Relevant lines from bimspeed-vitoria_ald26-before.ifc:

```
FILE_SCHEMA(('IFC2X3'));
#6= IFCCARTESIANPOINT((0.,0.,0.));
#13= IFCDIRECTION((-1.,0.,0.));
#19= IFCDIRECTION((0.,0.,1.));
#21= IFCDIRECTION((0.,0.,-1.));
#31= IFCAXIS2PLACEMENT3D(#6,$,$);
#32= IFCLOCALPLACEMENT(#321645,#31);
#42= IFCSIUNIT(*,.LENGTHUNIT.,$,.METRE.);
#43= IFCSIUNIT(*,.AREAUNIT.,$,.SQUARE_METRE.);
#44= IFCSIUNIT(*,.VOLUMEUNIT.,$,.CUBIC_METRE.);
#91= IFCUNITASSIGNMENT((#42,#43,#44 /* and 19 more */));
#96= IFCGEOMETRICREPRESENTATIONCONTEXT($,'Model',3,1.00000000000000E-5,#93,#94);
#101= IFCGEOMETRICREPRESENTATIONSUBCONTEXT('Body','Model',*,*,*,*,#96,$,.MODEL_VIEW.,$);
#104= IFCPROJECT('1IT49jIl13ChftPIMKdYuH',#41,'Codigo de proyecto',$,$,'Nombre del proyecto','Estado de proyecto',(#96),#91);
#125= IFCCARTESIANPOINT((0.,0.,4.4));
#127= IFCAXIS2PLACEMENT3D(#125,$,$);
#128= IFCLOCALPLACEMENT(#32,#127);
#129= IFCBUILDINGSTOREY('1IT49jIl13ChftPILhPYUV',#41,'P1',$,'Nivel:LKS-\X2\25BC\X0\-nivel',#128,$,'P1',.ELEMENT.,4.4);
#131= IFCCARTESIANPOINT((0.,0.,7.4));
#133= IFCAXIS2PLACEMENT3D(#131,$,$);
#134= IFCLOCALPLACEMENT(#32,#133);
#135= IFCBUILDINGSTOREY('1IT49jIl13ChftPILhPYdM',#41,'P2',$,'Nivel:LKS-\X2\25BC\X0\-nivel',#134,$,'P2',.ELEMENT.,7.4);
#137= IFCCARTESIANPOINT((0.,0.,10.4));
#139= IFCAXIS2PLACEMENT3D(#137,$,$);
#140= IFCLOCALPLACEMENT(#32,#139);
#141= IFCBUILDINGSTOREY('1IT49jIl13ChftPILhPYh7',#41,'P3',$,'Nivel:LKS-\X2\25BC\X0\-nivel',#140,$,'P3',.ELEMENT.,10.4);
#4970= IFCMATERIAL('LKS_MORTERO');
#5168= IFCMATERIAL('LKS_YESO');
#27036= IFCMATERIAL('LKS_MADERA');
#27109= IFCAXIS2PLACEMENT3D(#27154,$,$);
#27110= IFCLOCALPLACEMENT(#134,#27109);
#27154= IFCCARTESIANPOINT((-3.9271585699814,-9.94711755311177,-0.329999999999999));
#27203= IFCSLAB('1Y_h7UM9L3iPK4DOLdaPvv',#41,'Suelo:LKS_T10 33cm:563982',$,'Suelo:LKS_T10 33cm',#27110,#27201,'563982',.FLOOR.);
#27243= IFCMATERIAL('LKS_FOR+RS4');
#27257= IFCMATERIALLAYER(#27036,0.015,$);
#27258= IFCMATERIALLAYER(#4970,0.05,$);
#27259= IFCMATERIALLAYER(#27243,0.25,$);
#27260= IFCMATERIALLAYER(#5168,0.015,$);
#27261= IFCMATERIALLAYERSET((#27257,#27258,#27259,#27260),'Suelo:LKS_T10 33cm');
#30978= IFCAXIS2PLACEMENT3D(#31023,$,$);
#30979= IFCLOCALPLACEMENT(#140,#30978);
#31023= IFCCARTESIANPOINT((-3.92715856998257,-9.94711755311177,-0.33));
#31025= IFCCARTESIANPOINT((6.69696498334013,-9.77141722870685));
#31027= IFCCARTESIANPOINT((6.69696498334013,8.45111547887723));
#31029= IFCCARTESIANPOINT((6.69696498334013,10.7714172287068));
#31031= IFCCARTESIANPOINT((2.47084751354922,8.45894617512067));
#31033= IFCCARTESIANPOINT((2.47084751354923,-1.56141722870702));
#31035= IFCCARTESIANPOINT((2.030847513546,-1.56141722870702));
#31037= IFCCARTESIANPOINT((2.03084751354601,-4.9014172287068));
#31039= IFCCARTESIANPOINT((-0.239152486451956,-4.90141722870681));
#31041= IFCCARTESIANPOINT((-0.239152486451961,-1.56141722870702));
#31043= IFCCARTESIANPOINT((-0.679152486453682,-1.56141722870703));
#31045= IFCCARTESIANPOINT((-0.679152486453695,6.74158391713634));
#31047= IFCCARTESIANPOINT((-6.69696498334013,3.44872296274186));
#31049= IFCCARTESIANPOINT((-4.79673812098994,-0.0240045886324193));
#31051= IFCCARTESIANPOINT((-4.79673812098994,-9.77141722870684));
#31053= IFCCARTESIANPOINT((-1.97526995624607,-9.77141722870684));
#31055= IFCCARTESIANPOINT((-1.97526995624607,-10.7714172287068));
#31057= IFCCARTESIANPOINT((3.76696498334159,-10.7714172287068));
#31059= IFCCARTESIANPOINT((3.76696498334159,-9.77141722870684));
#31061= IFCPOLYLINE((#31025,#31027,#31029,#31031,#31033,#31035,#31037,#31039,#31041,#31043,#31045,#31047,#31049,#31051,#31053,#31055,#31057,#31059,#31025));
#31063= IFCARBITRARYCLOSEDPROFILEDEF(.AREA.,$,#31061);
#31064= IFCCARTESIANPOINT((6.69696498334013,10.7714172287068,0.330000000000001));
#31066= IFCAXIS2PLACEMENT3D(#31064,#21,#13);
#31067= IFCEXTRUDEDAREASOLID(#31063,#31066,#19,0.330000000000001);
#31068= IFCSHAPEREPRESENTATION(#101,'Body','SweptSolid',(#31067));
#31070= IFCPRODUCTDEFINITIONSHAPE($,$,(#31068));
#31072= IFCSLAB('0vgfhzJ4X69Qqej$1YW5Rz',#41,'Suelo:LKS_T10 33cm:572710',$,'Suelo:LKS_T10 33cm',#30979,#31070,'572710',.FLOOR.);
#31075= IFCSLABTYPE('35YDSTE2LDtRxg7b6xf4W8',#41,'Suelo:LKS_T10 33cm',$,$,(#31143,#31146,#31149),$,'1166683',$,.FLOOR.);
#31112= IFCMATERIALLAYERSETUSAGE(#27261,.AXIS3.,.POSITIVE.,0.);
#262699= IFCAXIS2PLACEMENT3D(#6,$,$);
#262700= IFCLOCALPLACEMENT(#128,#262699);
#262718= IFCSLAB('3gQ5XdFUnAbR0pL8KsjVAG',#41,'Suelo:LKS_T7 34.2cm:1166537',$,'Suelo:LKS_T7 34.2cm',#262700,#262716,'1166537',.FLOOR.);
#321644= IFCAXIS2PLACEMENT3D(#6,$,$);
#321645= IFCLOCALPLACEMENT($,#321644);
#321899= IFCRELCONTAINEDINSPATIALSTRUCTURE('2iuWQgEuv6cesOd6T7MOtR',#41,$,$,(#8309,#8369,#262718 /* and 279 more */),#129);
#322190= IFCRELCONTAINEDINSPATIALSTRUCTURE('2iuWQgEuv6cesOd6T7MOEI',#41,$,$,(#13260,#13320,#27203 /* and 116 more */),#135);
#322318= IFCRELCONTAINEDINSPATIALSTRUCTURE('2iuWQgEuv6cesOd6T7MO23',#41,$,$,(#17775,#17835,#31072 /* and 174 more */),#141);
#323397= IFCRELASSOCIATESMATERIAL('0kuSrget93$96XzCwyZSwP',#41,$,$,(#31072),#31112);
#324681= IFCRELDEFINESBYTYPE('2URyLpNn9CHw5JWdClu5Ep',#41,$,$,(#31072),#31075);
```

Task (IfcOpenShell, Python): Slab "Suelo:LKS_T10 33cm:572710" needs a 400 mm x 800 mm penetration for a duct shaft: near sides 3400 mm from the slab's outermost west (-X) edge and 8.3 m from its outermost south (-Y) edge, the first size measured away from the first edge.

```python
import numpy as np
import ifcopenshell
import ifcopenshell.api.feature
import ifcopenshell.api.geometry
import ifcopenshell.api.root
import ifcopenshell.geom
import ifcopenshell.util.placement
import ifcopenshell.util.representation
import ifcopenshell.util.shape
import ifcopenshell.util.unit

model = ifcopenshell.open("bimspeed-vitoria_ald26-before.ifc")
unit_scale = ifcopenshell.util.unit.calculate_unit_scale(model)
settings = ifcopenshell.geom.settings()


def volume(element):
    """Net volume in cubic metres, openings subtracted."""
    shape = ifcopenshell.geom.create_shape(settings, element)
    return ifcopenshell.util.shape.get_volume(shape.geometry)


slab = model.by_id(31072)
before = volume(slab)

# Extent in the slab's own axes, in metres. The edges named are its -X and -Y sides.
slab_shape = ifcopenshell.geom.create_shape(settings, slab)
vertices = ifcopenshell.util.shape.get_vertices(slab_shape.geometry)
x_min, y_min, bottom = vertices.min(axis=0)
top = vertices[:, 2].max()

opening = ifcopenshell.api.root.create_entity(model, ifc_class="IfcOpeningElement", name="Duct shaft opening")
context = ifcopenshell.util.representation.get_context(model, "Model", "Body", "MODEL_VIEW")
width, depth = 0.4, 0.8
outline = [(0.0, 0.0), (width, 0.0), (width, depth), (0.0, depth), (0.0, 0.0)]
# Overshoot both faces by 50 mm so the cut is clean.
shape = ifcopenshell.api.geometry.add_slab_representation(
    model, context=context, depth=top - bottom + 0.1, polyline=outline
)
ifcopenshell.api.geometry.assign_representation(model, product=opening, representation=shape)

matrix = ifcopenshell.util.placement.get_local_placement(slab.ObjectPlacement)
matrix[:, 3] = matrix @ np.append(np.array([x_min + 3.4, y_min + 8.3, bottom - 0.05]) / unit_scale, 1.0)
ifcopenshell.api.geometry.edit_object_placement(model, product=opening, matrix=matrix, is_si=False)
ifcopenshell.api.feature.add_feature(model, feature=opening, element=slab)

after = volume(slab)

print(f"slab volume {before:.3f} -> {after:.3f} m3")

model.write("bimspeed-vitoria_ald26-before-out.ifc")
```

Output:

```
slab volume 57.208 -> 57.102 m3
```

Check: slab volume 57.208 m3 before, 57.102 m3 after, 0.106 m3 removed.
